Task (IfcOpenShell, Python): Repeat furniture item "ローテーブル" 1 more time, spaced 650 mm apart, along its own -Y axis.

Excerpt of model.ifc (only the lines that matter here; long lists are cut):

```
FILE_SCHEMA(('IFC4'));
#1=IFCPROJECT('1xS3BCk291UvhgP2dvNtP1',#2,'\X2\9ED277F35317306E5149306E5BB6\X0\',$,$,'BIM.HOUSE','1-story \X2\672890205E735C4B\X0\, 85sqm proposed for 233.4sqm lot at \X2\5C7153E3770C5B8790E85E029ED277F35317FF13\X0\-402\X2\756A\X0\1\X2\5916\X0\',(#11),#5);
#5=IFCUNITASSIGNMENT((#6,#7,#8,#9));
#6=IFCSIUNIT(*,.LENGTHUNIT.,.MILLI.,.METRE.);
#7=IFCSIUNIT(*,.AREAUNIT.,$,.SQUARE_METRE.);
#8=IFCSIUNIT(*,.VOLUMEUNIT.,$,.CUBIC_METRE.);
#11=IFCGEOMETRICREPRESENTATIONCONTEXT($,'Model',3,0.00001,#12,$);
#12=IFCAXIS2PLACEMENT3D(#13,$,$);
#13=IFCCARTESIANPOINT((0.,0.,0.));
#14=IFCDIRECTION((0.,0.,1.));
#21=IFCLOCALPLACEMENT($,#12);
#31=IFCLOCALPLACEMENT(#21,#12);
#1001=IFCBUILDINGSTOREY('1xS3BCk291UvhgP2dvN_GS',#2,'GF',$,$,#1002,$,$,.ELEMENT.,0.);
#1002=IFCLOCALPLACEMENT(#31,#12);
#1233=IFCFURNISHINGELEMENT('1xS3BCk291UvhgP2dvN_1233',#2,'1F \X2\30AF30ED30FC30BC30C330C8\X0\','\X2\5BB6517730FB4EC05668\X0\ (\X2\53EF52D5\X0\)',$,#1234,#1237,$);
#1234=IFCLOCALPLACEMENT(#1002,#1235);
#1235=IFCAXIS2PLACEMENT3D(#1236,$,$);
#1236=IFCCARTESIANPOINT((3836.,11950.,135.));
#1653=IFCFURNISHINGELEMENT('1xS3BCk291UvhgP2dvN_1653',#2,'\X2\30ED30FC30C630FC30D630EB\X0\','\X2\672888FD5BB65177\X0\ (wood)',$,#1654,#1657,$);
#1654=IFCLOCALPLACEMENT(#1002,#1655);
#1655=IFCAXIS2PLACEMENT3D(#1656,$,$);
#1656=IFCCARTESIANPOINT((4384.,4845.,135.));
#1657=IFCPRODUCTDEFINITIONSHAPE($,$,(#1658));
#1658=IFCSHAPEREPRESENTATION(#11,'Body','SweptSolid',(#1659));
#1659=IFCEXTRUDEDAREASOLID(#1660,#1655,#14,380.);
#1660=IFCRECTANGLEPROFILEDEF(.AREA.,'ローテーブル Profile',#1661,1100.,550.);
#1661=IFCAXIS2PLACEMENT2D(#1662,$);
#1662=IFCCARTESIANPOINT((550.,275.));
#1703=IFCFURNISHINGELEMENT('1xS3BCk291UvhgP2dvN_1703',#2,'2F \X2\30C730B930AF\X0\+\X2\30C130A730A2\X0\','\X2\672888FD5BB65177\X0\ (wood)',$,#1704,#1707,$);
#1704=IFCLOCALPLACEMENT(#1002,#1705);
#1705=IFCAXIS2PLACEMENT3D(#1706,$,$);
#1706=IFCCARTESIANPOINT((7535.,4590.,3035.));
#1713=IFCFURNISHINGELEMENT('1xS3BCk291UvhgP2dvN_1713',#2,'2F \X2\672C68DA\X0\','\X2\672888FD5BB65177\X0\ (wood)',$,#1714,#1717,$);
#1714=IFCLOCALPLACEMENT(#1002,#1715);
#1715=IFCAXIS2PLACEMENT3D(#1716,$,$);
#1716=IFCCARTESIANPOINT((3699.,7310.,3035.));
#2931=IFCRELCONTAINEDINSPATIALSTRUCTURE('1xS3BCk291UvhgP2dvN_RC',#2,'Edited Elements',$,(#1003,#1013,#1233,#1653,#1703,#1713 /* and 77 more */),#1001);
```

```python
import ifcopenshell
import ifcopenshell.api.geometry
import ifcopenshell.api.root
import ifcopenshell.util.element
import ifcopenshell.util.placement
import ifcopenshell.util.unit

model = ifcopenshell.open("model.ifc")
unit_scale = ifcopenshell.util.unit.calculate_unit_scale(model)


def reuse_history(source, copy):
    """copy_class also copies each property set's owner history, people and application; keep the originals."""
    for rel in copy.IsDefinedBy:
        if rel.is_a("IfcRelDefinesByProperties") and (history := rel.RelatingPropertyDefinition.OwnerHistory):
            rel.RelatingPropertyDefinition.OwnerHistory = source.OwnerHistory
            ifcopenshell.util.element.remove_deep2(model, history)


source = model.by_guid("1xS3BCk291UvhgP2dvN_1653")
base = ifcopenshell.util.placement.get_local_placement(source.ObjectPlacement)
step = -base[:3, 1] * 0.65 / unit_scale

for i in range(1, 2):
    copy = ifcopenshell.api.root.copy_class(model, product=source)
    copy.Representation = ifcopenshell.util.element.copy_deep(
        model, source.Representation, exclude=["IfcGeometricRepresentationContext", "IfcRepresentationMap"]
    )
    reuse_history(source, copy)
    matrix = base.copy()
    matrix[:3, 3] += i * step
    print("added at", matrix[:3, 3].round(3) + 0.0)
    ifcopenshell.api.geometry.edit_object_placement(model, product=copy, matrix=matrix, is_si=False)

model.write("model_updated.ifc")
```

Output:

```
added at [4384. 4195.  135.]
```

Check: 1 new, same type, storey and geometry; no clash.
